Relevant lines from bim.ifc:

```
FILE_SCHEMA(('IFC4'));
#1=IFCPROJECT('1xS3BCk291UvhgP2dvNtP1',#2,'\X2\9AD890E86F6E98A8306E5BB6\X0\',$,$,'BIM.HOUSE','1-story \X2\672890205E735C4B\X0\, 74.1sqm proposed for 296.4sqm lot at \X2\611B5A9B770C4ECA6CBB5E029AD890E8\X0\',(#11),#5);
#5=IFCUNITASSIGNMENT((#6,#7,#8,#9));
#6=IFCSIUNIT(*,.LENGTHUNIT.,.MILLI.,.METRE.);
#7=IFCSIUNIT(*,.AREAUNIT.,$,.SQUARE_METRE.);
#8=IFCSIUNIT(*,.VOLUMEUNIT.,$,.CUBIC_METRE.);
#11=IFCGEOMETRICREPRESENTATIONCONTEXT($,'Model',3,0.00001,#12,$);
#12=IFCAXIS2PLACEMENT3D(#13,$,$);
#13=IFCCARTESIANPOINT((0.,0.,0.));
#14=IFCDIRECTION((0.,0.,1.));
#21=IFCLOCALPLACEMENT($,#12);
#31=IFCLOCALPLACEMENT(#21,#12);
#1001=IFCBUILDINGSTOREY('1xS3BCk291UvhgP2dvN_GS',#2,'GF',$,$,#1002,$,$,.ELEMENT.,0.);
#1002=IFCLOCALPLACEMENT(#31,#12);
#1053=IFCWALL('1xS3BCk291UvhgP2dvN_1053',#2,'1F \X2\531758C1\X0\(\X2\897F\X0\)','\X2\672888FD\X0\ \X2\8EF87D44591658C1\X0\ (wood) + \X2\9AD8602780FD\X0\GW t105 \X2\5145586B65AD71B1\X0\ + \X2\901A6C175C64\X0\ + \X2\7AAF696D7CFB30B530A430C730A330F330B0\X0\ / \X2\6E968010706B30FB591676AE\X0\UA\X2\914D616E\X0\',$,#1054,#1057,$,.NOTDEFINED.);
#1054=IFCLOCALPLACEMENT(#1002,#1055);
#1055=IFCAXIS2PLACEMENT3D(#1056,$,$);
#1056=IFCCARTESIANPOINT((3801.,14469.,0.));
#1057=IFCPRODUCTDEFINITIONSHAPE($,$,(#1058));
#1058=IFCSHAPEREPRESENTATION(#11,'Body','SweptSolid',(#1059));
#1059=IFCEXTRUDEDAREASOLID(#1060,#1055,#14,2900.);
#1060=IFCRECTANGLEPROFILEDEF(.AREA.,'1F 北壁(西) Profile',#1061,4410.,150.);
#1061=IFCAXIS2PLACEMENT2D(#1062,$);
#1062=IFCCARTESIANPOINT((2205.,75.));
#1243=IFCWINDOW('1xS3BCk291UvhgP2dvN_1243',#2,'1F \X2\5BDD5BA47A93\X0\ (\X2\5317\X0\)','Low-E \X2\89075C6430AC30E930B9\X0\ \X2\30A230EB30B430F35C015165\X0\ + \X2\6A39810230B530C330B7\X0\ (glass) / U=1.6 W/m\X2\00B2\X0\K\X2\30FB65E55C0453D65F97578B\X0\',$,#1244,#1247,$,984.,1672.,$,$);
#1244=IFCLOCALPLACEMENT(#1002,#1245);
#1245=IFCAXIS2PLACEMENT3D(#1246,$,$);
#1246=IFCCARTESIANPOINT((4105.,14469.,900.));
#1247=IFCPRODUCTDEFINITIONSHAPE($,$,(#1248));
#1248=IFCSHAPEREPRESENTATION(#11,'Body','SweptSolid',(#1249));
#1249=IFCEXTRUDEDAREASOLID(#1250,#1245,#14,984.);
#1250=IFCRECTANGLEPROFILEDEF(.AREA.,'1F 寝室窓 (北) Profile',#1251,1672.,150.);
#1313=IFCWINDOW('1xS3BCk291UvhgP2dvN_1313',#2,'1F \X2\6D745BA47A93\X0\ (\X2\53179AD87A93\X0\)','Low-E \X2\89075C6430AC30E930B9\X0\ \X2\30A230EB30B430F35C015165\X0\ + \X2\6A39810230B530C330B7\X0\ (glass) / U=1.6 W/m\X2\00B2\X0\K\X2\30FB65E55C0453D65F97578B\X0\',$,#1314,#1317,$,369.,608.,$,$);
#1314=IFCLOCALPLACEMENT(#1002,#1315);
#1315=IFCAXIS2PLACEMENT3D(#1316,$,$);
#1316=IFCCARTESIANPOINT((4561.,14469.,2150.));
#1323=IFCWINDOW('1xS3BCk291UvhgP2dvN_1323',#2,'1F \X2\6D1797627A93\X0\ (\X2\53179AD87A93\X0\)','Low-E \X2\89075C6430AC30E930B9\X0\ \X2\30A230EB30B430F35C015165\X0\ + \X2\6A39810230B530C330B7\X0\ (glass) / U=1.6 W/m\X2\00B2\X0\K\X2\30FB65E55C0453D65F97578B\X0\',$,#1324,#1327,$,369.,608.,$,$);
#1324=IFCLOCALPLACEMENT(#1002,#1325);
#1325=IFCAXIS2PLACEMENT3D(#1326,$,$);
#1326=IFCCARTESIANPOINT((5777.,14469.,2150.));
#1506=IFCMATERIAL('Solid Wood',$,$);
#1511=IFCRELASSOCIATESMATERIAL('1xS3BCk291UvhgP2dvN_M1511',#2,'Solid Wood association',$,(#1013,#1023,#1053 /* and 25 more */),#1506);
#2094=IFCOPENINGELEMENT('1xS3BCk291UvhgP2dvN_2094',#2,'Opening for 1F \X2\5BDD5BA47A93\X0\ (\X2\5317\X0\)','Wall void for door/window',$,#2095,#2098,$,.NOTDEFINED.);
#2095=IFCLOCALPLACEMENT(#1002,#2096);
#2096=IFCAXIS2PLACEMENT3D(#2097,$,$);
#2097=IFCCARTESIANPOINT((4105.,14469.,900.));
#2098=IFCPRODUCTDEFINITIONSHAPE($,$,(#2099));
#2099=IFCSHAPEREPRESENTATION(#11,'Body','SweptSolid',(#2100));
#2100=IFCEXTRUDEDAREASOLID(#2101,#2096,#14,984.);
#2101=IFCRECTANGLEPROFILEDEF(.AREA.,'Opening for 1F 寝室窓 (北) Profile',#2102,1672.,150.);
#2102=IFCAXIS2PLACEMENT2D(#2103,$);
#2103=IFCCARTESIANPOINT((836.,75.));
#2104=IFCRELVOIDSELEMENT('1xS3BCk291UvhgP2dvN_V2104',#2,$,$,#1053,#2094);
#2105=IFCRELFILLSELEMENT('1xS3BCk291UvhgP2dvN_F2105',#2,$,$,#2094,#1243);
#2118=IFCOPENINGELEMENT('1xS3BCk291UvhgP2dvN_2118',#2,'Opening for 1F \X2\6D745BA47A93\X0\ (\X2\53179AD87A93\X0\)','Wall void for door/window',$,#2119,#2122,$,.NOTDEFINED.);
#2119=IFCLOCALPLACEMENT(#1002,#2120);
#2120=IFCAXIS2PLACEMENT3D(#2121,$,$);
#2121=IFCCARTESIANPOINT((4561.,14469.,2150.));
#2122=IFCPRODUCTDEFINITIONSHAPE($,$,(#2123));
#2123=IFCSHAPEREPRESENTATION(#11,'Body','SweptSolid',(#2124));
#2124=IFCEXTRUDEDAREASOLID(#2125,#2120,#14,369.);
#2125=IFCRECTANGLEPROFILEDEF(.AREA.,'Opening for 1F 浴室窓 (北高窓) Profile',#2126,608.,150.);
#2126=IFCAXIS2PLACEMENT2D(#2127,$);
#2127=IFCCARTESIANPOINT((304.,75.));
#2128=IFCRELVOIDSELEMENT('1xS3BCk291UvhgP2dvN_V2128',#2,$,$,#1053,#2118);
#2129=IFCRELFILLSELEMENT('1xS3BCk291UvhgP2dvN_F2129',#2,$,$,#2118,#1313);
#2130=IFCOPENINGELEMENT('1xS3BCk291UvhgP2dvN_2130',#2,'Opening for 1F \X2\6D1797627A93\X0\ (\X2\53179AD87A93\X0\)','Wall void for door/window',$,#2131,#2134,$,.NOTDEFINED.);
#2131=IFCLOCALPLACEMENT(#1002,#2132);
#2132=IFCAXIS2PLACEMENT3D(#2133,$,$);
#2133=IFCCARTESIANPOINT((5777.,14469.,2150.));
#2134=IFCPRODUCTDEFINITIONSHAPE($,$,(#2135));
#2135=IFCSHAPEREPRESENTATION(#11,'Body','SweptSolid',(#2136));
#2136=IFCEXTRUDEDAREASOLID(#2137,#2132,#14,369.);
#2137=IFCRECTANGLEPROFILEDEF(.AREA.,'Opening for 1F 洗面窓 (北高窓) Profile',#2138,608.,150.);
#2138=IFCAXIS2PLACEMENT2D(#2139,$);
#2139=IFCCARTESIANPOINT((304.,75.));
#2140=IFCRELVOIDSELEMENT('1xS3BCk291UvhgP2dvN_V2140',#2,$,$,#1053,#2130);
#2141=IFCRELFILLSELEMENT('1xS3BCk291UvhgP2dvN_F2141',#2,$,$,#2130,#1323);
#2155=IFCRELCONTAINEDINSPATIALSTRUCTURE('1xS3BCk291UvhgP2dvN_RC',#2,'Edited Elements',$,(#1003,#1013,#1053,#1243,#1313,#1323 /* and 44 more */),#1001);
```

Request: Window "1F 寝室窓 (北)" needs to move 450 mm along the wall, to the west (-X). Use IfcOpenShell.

```python
import ifcopenshell
import ifcopenshell.api.geometry
import ifcopenshell.util.placement

model = ifcopenshell.open("bim.ifc")

window = model.by_guid("1xS3BCk291UvhgP2dvN_1243")
opening = window.FillsVoids[0].RelatingOpeningElement
wall = opening.VoidsElements[0].RelatingBuildingElement

wall_matrix = ifcopenshell.util.placement.get_local_placement(wall.ObjectPlacement)
shift = wall_matrix[:3, 0] * -450.0
before = ifcopenshell.util.placement.get_local_placement(window.ObjectPlacement)[:3, 3].copy()

# The window is not placed relative to its opening, so move both.
for product in (opening, window):
    matrix = ifcopenshell.util.placement.get_local_placement(product.ObjectPlacement)
    matrix[:3, 3] += shift
    ifcopenshell.api.geometry.edit_object_placement(model, product=product, matrix=matrix, is_si=False)

after = ifcopenshell.util.placement.get_local_placement(window.ObjectPlacement)[:3, 3]
print("window moved by", (after - before).round(3) + 0.0)

model.write("bim-out.ifc")
```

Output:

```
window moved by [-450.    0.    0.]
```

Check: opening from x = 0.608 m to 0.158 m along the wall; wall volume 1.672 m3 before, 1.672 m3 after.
